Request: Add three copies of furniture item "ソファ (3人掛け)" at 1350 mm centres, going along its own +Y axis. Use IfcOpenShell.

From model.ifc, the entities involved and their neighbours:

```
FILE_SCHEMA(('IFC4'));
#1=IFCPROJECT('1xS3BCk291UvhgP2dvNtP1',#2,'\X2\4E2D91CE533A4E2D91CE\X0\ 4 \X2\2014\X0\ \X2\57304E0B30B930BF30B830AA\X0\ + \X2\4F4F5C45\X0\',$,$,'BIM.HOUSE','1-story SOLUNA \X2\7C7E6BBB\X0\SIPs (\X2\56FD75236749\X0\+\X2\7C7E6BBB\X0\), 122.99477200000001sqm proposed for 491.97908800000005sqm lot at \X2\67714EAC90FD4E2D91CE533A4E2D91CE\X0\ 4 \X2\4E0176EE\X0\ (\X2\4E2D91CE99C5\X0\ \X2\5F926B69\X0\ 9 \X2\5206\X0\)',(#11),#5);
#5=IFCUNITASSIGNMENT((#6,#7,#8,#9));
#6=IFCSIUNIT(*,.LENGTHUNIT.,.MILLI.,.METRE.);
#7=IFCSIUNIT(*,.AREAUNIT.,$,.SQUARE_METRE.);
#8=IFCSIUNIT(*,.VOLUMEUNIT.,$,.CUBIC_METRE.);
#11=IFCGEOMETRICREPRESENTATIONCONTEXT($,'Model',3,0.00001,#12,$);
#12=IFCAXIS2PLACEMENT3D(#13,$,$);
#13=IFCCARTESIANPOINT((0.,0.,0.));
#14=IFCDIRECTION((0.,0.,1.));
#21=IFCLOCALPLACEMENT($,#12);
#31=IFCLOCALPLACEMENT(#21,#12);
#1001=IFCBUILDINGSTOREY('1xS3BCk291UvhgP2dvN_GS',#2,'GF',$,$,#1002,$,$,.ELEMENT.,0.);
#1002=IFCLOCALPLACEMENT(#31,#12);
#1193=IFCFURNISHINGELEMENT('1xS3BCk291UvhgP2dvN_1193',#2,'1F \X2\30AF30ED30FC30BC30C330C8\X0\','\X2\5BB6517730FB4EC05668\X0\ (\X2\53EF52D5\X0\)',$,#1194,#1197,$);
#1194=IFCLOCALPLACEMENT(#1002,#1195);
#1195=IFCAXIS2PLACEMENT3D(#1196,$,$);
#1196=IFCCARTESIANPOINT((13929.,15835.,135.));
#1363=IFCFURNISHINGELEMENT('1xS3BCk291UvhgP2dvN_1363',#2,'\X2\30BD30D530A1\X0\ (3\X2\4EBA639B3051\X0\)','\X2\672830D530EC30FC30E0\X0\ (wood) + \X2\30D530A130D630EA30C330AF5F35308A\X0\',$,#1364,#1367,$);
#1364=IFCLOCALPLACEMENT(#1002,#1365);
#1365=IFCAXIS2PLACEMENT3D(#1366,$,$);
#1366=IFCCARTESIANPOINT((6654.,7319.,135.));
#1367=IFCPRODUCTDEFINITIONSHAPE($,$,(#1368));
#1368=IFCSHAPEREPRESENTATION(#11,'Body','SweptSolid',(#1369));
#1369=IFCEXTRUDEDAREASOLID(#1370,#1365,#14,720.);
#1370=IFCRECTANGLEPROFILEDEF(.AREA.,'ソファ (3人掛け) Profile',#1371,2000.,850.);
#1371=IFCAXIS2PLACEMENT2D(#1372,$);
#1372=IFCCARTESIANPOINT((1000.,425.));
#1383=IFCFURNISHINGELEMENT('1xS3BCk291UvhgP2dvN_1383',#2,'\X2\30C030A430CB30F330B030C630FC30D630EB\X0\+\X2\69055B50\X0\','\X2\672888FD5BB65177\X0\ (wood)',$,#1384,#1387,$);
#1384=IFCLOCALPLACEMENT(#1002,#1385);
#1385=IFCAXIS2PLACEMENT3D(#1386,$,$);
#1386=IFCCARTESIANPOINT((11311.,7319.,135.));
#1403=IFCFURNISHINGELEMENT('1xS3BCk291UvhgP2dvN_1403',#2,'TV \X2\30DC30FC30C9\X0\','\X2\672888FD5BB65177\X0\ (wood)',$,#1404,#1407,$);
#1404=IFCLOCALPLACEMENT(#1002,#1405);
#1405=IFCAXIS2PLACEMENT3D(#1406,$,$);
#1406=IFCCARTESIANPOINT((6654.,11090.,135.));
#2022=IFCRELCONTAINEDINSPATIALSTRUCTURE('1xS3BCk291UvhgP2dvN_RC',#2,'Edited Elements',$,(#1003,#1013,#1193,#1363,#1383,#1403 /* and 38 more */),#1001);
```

```python
import ifcopenshell
import ifcopenshell.api.geometry
import ifcopenshell.api.root
import ifcopenshell.util.element
import ifcopenshell.util.placement
import ifcopenshell.util.unit

model = ifcopenshell.open("model.ifc")
unit_scale = ifcopenshell.util.unit.calculate_unit_scale(model)


def reuse_history(source, copy):
    """copy_class also copies each property set's owner history, people and application; keep the originals."""
    for rel in copy.IsDefinedBy:
        if rel.is_a("IfcRelDefinesByProperties") and (history := rel.RelatingPropertyDefinition.OwnerHistory):
            rel.RelatingPropertyDefinition.OwnerHistory = source.OwnerHistory
            ifcopenshell.util.element.remove_deep2(model, history)


source = model.by_guid("1xS3BCk291UvhgP2dvN_1363")
base = ifcopenshell.util.placement.get_local_placement(source.ObjectPlacement)
step = base[:3, 1] * 1.35 / unit_scale

for i in range(1, 4):
    copy = ifcopenshell.api.root.copy_class(model, product=source)
    copy.Representation = ifcopenshell.util.element.copy_deep(
        model, source.Representation, exclude=["IfcGeometricRepresentationContext", "IfcRepresentationMap"]
    )
    reuse_history(source, copy)
    matrix = base.copy()
    matrix[:3, 3] += i * step
    print("added at", matrix[:3, 3].round(3) + 0.0)
    ifcopenshell.api.geometry.edit_object_placement(model, product=copy, matrix=matrix, is_si=False)

model.write("model_edited.ifc")
```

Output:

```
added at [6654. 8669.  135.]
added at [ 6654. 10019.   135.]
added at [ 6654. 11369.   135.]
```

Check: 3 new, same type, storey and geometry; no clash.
